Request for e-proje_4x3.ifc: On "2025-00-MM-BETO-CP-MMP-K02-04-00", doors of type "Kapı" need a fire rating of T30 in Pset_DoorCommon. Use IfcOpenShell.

First a look at what the model holds.

```python
import ifcopenshell
import ifcopenshell.util.element

model = ifcopenshell.open("e-proje_4x3.ifc")
print(model.schema)
storey = next(s for s in model.by_type("IfcBuildingStorey") if s.Name == "2025-00-MM-BETO-CP-MMP-K02-04-00")
doors = [e for e in ifcopenshell.util.element.get_decomposition(storey) if e.is_a("IfcDoor")]
seen = {}
for e in doors:
    element_type = ifcopenshell.util.element.get_type(e)
    key = (element_type.Name if element_type != e and element_type else None, ifcopenshell.util.element.get_pset(e, "Pset_DoorCommon", "FireRating"))
    seen[key] = seen.get(key, 0) + 1
for (name, value), count in sorted(seen.items(), key=str):
    print(count, "x", name, "|", value)
```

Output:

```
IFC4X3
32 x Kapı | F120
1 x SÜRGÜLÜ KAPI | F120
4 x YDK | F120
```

```python
import ifcopenshell
import ifcopenshell.api.pset
import ifcopenshell.util.element

model = ifcopenshell.open("e-proje_4x3.ifc")

storey = next(s for s in model.by_type("IfcBuildingStorey") if s.Name == "2025-00-MM-BETO-CP-MMP-K02-04-00")
doors = [e for e in ifcopenshell.util.element.get_decomposition(storey) if e.is_a("IfcDoor")]

count = 0
for e in doors:
    element_type = ifcopenshell.util.element.get_type(e)
    if element_type in (None, e) or element_type.Name != "Kapı":
        continue
    # add_pset returns the element's existing set when there is one.
    pset = ifcopenshell.api.pset.add_pset(model, product=e, name="Pset_DoorCommon")
    ifcopenshell.api.pset.edit_pset(model, pset=pset, properties={"FireRating": "T30"})
    count += 1

print(count, "doors updated")

model.write("e-proje_4x3_edited.ifc")
```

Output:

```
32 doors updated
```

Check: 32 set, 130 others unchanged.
